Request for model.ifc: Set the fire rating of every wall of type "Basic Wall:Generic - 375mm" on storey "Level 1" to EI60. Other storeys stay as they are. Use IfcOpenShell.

First a look at what the model holds.

```python
import ifcopenshell
import ifcopenshell.util.element

model = ifcopenshell.open("model.ifc")
print(model.schema)
storey = next(s for s in model.by_type("IfcBuildingStorey") if s.Name == "Level 1")
walls = [e for e in ifcopenshell.util.element.get_decomposition(storey) if e.is_a("IfcWall")]
seen = {}
for e in walls:
    element_type = ifcopenshell.util.element.get_type(e)
    key = (element_type.Name if element_type != e and element_type else None, ifcopenshell.util.element.get_pset(e, "Pset_WallCommon", "FireRating"))
    seen[key] = seen.get(key, 0) + 1
for (name, value), count in sorted(seen.items(), key=str):
    print(count, "x", name, "|", value)
```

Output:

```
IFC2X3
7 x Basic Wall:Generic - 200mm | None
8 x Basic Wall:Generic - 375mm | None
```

```python
import ifcopenshell
import ifcopenshell.api.pset
import ifcopenshell.util.element

model = ifcopenshell.open("model.ifc")

storey = next(s for s in model.by_type("IfcBuildingStorey") if s.Name == "Level 1")
walls = [e for e in ifcopenshell.util.element.get_decomposition(storey) if e.is_a("IfcWall")]

count = 0
for e in walls:
    element_type = ifcopenshell.util.element.get_type(e)
    if element_type in (None, e) or element_type.Name != "Basic Wall:Generic - 375mm":
        continue
    # add_pset returns the element's existing set when there is one.
    pset = ifcopenshell.api.pset.add_pset(model, product=e, name="Pset_WallCommon")
    ifcopenshell.api.pset.edit_pset(model, pset=pset, properties={"FireRating": "EI60"})
    count += 1

print(count, "walls updated")

model.write("model_rev.ifc")
```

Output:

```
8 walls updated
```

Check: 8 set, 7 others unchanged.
